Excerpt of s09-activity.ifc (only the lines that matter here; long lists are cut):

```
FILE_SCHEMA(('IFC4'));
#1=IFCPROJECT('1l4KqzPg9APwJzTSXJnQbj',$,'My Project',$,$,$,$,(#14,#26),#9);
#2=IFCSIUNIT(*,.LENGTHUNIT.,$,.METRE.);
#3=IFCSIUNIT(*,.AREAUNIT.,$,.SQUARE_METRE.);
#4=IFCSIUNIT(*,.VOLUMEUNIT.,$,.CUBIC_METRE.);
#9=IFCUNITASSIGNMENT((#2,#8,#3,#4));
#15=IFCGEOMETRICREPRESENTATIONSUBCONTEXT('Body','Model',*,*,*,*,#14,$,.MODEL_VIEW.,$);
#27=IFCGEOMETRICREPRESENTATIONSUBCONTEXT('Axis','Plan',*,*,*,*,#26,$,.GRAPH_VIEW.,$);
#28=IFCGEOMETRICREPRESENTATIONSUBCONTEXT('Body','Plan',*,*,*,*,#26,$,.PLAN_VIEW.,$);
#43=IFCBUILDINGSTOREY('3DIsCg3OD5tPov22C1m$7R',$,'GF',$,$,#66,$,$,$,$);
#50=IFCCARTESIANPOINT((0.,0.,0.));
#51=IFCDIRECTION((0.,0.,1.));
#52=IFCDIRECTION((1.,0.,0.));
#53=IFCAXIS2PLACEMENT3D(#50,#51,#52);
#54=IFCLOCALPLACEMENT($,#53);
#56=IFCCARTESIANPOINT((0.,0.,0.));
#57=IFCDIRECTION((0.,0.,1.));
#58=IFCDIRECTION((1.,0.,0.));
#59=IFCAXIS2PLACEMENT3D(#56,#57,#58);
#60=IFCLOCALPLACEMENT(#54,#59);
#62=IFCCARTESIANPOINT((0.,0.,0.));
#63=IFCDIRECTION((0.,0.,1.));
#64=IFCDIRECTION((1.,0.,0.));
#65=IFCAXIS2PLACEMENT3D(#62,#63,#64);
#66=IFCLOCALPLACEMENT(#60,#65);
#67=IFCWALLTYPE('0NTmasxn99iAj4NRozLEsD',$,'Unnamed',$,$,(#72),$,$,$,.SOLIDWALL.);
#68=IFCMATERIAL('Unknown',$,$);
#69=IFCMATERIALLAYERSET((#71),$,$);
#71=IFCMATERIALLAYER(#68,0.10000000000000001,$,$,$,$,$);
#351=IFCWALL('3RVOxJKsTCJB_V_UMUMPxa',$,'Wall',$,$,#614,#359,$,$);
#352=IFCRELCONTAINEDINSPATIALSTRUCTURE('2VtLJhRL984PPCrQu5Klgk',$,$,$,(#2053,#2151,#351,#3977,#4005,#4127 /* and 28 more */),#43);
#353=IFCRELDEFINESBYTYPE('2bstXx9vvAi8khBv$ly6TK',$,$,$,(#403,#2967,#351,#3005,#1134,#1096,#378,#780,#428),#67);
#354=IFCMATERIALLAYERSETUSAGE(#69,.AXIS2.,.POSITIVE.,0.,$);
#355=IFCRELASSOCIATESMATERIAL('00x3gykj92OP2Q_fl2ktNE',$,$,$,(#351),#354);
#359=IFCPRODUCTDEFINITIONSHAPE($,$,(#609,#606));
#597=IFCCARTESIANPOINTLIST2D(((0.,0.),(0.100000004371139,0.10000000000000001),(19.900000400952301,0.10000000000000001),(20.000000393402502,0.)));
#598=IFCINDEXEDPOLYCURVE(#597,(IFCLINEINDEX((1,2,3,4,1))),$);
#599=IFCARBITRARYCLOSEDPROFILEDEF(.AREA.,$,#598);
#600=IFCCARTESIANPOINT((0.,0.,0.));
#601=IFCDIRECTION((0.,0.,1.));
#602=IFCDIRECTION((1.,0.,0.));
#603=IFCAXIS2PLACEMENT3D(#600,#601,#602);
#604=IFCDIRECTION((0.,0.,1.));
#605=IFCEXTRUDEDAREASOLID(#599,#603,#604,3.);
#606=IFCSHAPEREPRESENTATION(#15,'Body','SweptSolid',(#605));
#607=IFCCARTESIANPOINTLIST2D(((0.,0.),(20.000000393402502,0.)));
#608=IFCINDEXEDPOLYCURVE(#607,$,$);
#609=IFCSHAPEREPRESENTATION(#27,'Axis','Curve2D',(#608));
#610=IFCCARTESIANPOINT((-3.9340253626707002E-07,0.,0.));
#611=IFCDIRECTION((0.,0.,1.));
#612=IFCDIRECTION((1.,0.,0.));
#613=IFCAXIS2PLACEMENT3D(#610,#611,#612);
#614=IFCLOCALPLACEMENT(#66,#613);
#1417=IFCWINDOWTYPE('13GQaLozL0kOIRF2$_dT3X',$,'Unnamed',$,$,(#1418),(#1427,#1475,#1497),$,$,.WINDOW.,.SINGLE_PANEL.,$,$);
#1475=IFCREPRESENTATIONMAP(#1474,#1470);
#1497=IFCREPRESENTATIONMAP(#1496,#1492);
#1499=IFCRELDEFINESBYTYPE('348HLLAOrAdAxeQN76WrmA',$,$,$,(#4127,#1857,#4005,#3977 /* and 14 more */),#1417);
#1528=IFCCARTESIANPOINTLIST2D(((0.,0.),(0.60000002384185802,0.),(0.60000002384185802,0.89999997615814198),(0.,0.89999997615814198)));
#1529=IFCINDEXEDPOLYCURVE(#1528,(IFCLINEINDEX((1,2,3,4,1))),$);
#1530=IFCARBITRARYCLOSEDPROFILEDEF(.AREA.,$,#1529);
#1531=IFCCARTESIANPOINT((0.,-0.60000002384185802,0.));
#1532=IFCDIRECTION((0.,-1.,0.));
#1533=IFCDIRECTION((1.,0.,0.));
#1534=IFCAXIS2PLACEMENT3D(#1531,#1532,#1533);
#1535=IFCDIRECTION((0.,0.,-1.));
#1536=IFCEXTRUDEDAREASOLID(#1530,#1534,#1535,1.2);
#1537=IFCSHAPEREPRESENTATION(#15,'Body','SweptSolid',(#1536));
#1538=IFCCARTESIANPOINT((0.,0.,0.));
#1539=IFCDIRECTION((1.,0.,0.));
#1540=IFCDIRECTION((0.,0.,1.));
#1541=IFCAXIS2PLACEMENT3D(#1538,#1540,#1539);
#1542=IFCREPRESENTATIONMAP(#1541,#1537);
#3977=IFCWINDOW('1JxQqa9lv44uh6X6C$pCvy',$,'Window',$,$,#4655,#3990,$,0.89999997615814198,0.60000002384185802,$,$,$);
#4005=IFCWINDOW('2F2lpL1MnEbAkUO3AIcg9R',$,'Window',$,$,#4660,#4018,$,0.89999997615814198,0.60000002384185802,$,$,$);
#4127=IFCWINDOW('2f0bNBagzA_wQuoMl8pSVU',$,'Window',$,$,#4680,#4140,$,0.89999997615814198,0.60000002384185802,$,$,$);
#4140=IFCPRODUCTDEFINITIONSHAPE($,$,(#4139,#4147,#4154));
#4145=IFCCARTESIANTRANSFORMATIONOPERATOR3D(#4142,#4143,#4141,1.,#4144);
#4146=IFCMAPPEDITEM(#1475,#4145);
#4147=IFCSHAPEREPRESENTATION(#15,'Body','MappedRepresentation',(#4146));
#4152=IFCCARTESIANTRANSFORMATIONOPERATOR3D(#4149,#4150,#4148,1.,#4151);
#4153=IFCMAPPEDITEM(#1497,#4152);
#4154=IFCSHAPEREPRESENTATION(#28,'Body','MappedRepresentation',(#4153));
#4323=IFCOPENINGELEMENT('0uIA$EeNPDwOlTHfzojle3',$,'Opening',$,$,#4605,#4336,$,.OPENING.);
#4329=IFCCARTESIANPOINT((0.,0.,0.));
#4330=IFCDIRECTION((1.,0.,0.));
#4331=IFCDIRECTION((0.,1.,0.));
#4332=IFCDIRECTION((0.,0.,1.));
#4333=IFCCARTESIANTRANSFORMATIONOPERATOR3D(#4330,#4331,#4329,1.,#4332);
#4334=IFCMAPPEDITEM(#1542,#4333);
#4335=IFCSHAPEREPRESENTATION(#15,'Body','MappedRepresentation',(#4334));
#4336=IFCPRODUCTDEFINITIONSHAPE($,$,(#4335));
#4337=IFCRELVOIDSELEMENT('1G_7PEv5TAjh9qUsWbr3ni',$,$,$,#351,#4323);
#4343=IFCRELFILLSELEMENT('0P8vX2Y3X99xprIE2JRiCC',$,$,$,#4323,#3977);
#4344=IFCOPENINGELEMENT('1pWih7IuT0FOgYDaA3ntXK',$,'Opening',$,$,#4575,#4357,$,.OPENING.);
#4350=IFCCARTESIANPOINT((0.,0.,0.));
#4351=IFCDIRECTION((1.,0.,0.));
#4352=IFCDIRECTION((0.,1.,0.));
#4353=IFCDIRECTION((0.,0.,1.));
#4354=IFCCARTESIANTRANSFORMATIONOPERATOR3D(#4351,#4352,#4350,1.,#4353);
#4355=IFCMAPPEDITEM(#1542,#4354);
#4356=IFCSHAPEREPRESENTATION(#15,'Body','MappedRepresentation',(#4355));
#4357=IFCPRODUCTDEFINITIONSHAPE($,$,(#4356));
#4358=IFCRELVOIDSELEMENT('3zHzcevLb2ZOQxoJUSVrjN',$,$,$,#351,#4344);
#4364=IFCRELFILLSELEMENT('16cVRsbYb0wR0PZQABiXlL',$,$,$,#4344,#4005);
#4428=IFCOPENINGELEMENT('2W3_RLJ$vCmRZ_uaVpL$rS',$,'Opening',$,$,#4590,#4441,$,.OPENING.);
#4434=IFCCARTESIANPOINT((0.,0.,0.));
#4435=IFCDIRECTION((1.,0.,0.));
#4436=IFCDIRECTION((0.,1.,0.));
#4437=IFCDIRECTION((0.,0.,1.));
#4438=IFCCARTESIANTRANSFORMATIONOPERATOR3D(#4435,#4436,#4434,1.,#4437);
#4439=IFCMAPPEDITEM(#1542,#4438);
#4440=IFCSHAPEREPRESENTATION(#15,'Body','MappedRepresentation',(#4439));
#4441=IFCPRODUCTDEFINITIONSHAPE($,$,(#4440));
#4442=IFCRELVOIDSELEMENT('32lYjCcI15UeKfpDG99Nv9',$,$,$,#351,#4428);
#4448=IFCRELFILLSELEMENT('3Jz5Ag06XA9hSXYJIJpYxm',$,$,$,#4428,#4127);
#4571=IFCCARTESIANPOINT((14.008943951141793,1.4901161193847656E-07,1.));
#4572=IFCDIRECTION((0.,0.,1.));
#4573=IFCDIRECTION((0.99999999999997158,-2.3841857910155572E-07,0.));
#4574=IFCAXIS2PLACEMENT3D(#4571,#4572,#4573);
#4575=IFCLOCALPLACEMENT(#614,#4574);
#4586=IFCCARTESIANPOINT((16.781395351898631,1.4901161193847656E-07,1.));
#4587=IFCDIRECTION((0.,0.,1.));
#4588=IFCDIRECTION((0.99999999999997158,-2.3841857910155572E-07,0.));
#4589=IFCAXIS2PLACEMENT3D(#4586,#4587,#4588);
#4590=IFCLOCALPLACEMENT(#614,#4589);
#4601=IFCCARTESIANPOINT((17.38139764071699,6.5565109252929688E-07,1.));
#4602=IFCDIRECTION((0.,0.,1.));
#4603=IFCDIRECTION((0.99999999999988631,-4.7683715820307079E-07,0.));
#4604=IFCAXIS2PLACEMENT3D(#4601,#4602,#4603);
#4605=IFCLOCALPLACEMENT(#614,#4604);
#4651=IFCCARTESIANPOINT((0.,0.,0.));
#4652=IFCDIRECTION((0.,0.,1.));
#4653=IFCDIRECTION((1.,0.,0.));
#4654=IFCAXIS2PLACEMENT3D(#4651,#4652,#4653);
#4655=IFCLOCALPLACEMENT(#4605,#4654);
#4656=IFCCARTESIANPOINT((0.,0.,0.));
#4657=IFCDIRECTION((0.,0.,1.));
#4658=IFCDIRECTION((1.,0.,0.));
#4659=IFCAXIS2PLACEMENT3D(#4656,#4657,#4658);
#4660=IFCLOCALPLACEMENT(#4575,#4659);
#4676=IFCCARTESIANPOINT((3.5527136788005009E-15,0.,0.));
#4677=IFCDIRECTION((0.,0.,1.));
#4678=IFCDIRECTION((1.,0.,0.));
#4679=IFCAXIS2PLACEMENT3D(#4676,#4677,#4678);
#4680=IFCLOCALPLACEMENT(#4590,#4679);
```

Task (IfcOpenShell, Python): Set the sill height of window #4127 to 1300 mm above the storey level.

```python
import numpy as np
import ifcopenshell
import ifcopenshell.api.geometry
import ifcopenshell.geom
import ifcopenshell.util.element
import ifcopenshell.util.placement
import ifcopenshell.util.shape
import ifcopenshell.util.unit

model = ifcopenshell.open("s09-activity.ifc")
unit_scale = ifcopenshell.util.unit.calculate_unit_scale(model)

window = model.by_guid("2f0bNBagzA_wQuoMl8pSVU")
opening = window.FillsVoids[0].RelatingOpeningElement
storey = ifcopenshell.util.element.get_container(window, ifc_class="IfcBuildingStorey")
level = ifcopenshell.util.placement.get_local_placement(storey.ObjectPlacement)[2, 3]

# The opening's origin need not be at the sill, so measure its lowest point.
shape = ifcopenshell.geom.create_shape(ifcopenshell.geom.settings(), opening)
bottom = ifcopenshell.util.shape.get_shape_bottom_elevation(shape, shape.geometry) / unit_scale
dz = level + 1.3 - bottom

shift = np.array([0.0, 0.0, dz])
# The window is placed relative to its opening, so it follows when the opening moves.
matrix = ifcopenshell.util.placement.get_local_placement(opening.ObjectPlacement)
matrix[:3, 3] += shift
ifcopenshell.api.geometry.edit_object_placement(
    model, product=opening, matrix=matrix, is_si=False, should_transform_children=True
)

print(f"moved by {dz * unit_scale:+.3f} m")

model.write("s09-activity-out.ifc")
```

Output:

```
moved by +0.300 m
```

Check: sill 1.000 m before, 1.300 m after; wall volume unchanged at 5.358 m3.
